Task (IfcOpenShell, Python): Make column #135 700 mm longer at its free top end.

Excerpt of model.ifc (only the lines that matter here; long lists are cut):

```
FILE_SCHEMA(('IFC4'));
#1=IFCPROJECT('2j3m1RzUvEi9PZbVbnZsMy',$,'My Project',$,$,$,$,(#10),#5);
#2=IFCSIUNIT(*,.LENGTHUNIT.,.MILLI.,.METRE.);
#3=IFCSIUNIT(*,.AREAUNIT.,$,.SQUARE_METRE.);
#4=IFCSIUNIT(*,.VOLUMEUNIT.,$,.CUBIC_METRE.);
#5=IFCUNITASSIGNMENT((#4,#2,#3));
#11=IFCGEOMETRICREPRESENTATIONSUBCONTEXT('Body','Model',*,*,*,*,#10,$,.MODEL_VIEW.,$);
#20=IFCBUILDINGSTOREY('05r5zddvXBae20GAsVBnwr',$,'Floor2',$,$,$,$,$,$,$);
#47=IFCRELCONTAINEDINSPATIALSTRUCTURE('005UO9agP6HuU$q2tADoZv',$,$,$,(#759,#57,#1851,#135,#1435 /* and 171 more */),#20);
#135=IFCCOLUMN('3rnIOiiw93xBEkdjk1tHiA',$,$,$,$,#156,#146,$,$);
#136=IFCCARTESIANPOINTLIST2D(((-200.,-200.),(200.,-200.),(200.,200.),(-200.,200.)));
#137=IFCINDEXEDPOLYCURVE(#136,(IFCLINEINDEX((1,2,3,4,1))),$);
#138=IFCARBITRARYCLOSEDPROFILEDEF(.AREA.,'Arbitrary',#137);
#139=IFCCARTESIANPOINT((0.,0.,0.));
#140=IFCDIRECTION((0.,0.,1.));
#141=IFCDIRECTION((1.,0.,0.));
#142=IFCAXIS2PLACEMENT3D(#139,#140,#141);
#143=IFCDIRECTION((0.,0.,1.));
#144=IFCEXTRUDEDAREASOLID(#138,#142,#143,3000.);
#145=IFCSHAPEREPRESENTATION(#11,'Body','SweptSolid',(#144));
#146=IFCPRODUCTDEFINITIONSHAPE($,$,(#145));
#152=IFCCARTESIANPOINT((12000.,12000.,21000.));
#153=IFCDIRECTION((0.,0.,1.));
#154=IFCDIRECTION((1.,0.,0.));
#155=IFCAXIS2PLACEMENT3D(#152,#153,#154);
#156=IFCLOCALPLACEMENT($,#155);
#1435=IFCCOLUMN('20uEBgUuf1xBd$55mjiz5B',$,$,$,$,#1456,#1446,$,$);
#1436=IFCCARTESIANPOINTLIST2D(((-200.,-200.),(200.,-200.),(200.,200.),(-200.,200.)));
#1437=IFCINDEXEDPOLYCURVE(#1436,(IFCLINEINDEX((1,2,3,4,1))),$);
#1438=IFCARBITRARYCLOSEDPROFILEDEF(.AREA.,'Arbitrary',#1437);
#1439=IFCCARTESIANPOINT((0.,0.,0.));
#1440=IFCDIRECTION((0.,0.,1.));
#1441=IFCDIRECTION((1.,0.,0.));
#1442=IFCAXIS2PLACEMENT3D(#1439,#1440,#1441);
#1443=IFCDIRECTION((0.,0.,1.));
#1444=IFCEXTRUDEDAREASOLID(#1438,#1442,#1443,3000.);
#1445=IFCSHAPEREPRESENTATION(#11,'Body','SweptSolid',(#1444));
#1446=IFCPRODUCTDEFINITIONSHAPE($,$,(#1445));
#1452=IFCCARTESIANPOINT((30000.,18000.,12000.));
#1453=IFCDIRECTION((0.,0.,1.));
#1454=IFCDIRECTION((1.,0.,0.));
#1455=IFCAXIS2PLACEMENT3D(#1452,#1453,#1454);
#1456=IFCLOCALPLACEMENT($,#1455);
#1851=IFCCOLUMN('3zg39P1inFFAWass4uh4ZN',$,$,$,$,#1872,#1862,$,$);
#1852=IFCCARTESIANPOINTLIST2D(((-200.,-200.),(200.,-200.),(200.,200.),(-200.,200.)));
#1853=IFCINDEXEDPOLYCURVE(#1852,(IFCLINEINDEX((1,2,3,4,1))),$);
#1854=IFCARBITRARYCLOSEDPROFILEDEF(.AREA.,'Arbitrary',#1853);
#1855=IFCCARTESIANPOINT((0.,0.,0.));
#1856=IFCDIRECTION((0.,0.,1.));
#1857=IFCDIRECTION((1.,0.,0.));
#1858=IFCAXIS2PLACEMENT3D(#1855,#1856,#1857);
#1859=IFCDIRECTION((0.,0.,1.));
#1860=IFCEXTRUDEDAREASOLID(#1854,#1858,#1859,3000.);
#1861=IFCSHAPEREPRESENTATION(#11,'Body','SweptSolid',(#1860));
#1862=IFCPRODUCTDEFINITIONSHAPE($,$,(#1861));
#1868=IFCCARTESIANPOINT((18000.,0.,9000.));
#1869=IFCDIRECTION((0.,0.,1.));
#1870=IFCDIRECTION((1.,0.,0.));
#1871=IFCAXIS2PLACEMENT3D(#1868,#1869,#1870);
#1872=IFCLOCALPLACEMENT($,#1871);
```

```python
import ifcopenshell
import ifcopenshell.util.representation
import ifcopenshell.util.unit

model = ifcopenshell.open("model.ifc")
unit_scale = ifcopenshell.util.unit.calculate_unit_scale(model)

member = model.by_id(135)
change = 0.7 / unit_scale

# The extrusion runs towards the end named, so only its depth changes.
body = ifcopenshell.util.representation.get_representation(member, "Model", "Body")
solid = body.Items[0]
old_length = solid.Depth
solid.Depth += change

print(f"length {old_length:g} -> {solid.Depth:g}")

model.write("model_v2.ifc")
```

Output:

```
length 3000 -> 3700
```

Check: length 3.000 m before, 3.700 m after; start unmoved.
